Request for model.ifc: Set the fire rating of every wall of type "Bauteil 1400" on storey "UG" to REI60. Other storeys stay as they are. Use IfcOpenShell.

First a look at what the model holds.

```python
import ifcopenshell
import ifcopenshell.util.element

model = ifcopenshell.open("model.ifc")
print(model.schema)
storey = next(s for s in model.by_type("IfcBuildingStorey") if s.Name == "UG")
walls = [e for e in ifcopenshell.util.element.get_decomposition(storey) if e.is_a("IfcWall")]
seen = {}
for e in walls:
    element_type = ifcopenshell.util.element.get_type(e)
    key = (element_type.Name if element_type != e and element_type else None, ifcopenshell.util.element.get_pset(e, "Pset_WallCommon", "FireRating"))
    seen[key] = seen.get(key, 0) + 1
for (name, value), count in sorted(seen.items(), key=str):
    print(count, "x", name, "|", value)
```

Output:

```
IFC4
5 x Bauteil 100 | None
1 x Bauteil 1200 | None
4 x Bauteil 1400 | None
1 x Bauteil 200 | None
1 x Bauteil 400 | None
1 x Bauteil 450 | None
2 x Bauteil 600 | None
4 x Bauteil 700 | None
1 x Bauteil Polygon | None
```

```python
import ifcopenshell
import ifcopenshell.api.pset
import ifcopenshell.util.element

model = ifcopenshell.open("model.ifc")

storey = next(s for s in model.by_type("IfcBuildingStorey") if s.Name == "UG")
walls = [e for e in ifcopenshell.util.element.get_decomposition(storey) if e.is_a("IfcWall")]

count = 0
for e in walls:
    element_type = ifcopenshell.util.element.get_type(e)
    if element_type in (None, e) or element_type.Name != "Bauteil 1400":
        continue
    # add_pset returns the element's existing set when there is one.
    pset = ifcopenshell.api.pset.add_pset(model, product=e, name="Pset_WallCommon")
    ifcopenshell.api.pset.edit_pset(model, pset=pset, properties={"FireRating": "REI60"})
    count += 1

print(count, "walls updated")

model.write("model_rev.ifc")
```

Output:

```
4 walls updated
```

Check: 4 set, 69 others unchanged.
